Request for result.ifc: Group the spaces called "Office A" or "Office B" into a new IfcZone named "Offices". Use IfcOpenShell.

First a look at what the model holds.

```python
import ifcopenshell

model = ifcopenshell.open("result.ifc")
print(model.schema)
seen = {}
for space in model.by_type("IfcSpace"):
    seen[space.Name] = seen.get(space.Name, 0) + 1
for name, count in sorted(seen.items(), key=str):
    print(count, "x", name)
print("zones:", [z.Name for z in model.by_type("IfcZone")][:20])
```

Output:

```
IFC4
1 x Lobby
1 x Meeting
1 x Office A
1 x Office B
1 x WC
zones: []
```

```python
import ifcopenshell
import ifcopenshell.api.group
import ifcopenshell.api.root

model = ifcopenshell.open("result.ifc")

names = {"Office A", "Office B"}
spaces = [s for s in model.by_type("IfcSpace") if s.Name in names]

zone = ifcopenshell.api.root.create_entity(model, ifc_class="IfcZone", name="Offices")
ifcopenshell.api.group.assign_group(model, products=spaces, group=zone)
print(len(spaces), "spaces in", zone.Name)

model.write("result_rev.ifc")
```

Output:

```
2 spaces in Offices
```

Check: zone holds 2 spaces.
